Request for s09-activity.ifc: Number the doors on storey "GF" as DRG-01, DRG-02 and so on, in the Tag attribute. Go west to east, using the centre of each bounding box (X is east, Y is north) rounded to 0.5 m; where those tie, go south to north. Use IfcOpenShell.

First a look at what the model holds.

```python
import ifcopenshell
import ifcopenshell.util.element
import ifcopenshell.util.placement

model = ifcopenshell.open("s09-activity.ifc")
print(model.schema)
storey = next(s for s in model.by_type("IfcBuildingStorey") if s.Name == "GF")
doors = [e for e in ifcopenshell.util.element.get_decomposition(storey) if e.is_a("IfcDoor")]
for e in sorted(doors, key=lambda e: e.id()):
    origin = ifcopenshell.util.placement.get_local_placement(e.ObjectPlacement)[:3, 3]
    print(e.id(), e.Tag, e.Name, origin.round(2) + 0.0, sep=" | ")
```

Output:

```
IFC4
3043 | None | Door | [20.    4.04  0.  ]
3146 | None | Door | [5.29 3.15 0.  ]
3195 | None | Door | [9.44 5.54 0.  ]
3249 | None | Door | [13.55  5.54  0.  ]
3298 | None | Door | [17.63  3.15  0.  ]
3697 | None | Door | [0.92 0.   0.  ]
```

```python
import ifcopenshell
import ifcopenshell.geom
import ifcopenshell.util.element
import ifcopenshell.util.shape

model = ifcopenshell.open("s09-activity.ifc")
settings = ifcopenshell.geom.settings()
settings.set("use-world-coords", True)


def centre(element):
    shape = ifcopenshell.geom.create_shape(settings, element)
    return ifcopenshell.util.shape.get_bbox_centroid(shape.geometry)


storey = next(s for s in model.by_type("IfcBuildingStorey") if s.Name == "GF")
doors = [e for e in ifcopenshell.util.element.get_decomposition(storey) if e.is_a("IfcDoor")]

# Insertion points can sit at a corner or the storey origin, so sort by the geometry (in metres).
centres = {e: centre(e) for e in doors}
doors.sort(key=lambda e: (round(centres[e][0] / 0.5), centres[e][1]))

for i, e in enumerate(doors, start=1):
    number = f"DRG-{i:02d}"
    e.Tag = number
    print(e.id(), number)

model.write("s09-activity_updated.ifc")
```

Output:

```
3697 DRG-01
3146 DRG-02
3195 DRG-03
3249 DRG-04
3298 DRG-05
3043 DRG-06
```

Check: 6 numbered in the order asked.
